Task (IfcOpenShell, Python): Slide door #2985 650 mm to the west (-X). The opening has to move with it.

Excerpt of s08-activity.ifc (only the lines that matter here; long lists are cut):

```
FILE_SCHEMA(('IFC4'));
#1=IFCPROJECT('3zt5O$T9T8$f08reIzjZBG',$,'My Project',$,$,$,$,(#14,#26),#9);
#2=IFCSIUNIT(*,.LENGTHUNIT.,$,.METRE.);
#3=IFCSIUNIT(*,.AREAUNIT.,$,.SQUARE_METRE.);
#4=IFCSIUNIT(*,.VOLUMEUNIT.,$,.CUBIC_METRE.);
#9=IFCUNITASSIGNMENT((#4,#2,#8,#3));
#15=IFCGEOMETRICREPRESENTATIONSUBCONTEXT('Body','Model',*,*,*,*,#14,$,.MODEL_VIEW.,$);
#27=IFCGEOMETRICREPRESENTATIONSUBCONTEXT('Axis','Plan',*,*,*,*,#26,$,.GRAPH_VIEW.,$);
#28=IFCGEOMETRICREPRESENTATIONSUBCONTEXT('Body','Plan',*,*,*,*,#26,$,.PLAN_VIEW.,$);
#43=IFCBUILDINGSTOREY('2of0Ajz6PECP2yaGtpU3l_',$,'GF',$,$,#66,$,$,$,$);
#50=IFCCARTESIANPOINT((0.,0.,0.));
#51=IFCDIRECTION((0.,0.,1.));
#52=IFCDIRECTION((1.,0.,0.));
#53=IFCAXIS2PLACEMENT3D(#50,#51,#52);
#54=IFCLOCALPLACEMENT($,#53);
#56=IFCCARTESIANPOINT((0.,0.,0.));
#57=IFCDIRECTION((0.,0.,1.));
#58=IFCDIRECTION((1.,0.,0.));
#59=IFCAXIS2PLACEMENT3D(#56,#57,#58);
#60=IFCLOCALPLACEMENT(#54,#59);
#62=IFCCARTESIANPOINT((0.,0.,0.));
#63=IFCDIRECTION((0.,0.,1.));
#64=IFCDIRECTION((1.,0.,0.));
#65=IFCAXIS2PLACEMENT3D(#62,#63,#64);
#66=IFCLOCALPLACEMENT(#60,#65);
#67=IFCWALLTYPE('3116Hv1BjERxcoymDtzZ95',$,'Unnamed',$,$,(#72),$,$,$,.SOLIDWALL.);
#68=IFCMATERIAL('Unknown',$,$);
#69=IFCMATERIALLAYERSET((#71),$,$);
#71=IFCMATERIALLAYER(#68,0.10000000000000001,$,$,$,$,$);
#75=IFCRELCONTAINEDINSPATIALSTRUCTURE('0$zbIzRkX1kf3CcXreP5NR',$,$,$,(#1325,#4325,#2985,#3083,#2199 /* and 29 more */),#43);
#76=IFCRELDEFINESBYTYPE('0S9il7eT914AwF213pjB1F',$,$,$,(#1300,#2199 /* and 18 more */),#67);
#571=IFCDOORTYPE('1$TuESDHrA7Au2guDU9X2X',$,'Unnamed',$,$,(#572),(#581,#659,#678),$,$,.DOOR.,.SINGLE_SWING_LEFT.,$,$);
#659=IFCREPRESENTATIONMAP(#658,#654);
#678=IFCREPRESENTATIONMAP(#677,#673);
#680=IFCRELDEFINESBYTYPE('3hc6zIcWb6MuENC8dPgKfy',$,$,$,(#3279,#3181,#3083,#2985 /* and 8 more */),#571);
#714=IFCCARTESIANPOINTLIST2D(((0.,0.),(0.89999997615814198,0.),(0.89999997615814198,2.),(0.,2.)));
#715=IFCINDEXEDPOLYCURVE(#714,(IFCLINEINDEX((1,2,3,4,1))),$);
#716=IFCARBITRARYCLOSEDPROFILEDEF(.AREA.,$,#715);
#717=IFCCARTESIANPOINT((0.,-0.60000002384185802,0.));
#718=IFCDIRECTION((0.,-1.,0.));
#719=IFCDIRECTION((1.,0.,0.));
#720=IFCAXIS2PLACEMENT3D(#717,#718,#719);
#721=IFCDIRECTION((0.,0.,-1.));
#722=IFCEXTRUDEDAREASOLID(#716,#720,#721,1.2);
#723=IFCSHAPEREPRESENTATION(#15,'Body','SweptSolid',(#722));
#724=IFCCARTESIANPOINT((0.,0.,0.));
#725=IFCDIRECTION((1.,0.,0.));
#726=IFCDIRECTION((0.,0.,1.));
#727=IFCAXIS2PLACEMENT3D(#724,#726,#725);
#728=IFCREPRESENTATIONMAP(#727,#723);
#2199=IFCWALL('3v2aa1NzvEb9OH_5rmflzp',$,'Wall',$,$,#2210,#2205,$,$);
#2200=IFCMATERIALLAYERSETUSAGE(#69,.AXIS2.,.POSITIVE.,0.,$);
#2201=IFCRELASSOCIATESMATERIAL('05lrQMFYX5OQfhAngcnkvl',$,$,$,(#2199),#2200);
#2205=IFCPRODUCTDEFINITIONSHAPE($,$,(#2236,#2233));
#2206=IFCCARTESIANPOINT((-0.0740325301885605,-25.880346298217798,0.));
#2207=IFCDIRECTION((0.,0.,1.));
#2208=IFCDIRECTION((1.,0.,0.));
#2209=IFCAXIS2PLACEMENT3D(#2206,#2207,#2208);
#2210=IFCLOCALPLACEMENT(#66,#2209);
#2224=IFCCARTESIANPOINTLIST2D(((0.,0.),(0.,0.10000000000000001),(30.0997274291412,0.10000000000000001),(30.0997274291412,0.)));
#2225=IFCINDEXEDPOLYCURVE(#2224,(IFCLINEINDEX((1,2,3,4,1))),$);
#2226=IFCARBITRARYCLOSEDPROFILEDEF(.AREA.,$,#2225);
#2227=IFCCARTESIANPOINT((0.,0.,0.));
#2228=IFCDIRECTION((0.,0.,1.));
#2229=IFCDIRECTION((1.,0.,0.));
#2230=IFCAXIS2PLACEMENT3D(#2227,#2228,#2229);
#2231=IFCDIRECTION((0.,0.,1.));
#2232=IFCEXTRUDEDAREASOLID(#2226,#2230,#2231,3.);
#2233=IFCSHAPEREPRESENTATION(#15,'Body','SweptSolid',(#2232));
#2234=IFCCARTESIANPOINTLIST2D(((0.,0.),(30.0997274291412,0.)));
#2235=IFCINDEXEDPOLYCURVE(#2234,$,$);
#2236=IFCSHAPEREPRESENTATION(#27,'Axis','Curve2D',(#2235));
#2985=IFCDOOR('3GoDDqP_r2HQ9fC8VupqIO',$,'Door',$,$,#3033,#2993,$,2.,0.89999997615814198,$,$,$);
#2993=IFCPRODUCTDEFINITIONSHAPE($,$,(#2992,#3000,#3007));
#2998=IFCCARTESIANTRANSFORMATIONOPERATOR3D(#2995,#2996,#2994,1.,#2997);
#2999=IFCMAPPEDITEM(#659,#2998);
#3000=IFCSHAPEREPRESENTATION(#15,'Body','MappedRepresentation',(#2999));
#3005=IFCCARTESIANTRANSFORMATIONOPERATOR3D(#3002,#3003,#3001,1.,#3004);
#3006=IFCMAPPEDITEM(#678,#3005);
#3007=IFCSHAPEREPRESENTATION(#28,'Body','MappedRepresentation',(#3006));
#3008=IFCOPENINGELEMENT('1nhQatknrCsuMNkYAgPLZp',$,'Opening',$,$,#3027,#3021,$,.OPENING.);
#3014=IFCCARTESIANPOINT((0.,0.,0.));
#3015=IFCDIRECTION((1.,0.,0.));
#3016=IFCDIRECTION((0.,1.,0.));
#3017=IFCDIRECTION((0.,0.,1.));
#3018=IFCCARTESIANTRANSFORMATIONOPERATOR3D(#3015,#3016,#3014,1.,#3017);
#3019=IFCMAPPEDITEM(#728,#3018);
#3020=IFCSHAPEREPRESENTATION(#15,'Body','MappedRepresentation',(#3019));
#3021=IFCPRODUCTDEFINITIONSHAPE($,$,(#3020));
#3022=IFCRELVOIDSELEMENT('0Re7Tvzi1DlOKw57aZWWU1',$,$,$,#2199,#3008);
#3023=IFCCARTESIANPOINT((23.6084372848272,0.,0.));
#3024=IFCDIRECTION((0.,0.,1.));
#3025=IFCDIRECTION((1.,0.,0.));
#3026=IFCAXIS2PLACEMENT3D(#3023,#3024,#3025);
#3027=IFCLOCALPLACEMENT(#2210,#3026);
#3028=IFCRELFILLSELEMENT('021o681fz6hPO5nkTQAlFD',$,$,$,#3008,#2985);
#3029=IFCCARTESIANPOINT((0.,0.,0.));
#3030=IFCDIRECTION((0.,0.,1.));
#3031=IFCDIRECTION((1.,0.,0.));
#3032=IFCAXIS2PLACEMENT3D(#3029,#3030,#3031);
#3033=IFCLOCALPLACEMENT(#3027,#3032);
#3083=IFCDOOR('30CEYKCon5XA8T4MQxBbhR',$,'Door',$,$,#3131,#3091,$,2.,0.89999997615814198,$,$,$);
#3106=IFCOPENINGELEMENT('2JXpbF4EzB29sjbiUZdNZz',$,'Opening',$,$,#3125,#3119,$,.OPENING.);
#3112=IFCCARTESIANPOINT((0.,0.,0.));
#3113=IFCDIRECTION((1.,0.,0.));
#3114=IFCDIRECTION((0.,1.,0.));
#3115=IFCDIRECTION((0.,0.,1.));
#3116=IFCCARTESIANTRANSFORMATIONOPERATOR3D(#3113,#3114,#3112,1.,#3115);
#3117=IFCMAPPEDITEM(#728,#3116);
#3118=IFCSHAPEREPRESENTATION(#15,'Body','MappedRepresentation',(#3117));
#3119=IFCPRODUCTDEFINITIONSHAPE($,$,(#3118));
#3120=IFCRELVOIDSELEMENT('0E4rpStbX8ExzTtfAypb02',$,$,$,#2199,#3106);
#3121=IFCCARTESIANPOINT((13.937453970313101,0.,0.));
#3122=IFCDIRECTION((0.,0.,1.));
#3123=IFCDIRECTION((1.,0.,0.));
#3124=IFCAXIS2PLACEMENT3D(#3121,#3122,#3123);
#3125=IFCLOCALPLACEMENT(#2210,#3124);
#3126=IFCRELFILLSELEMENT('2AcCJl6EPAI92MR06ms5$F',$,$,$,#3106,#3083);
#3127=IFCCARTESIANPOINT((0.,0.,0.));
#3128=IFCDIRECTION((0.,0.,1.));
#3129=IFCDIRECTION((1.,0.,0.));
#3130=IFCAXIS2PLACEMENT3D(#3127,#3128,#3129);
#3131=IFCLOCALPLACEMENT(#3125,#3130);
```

```python
import ifcopenshell
import ifcopenshell.api.geometry
import ifcopenshell.util.placement
import ifcopenshell.util.unit

model = ifcopenshell.open("s08-activity.ifc")
unit_scale = ifcopenshell.util.unit.calculate_unit_scale(model)

door = model.by_guid("3GoDDqP_r2HQ9fC8VupqIO")
opening = door.FillsVoids[0].RelatingOpeningElement
wall = opening.VoidsElements[0].RelatingBuildingElement

wall_matrix = ifcopenshell.util.placement.get_local_placement(wall.ObjectPlacement)
shift = wall_matrix[:3, 0] * -0.65 / unit_scale
before = ifcopenshell.util.placement.get_local_placement(door.ObjectPlacement)[:3, 3].copy()

# The door is placed relative to its opening, so it follows when the opening moves.
matrix = ifcopenshell.util.placement.get_local_placement(opening.ObjectPlacement)
matrix[:3, 3] += shift
ifcopenshell.api.geometry.edit_object_placement(
    model, product=opening, matrix=matrix, is_si=False, should_transform_children=True
)

after = ifcopenshell.util.placement.get_local_placement(door.ObjectPlacement)[:3, 3]
print("door moved by", (after - before).round(3) + 0.0)

model.write("s08-activity_updated.ifc")
```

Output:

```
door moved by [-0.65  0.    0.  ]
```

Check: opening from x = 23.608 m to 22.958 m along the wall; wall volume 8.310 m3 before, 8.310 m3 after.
